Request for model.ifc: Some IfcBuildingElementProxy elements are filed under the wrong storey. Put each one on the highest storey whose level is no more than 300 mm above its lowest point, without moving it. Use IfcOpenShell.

First a look at what the model holds.

```python
import ifcopenshell
import ifcopenshell.util.element
import ifcopenshell.util.placement

model = ifcopenshell.open("model.ifc")
print(model.schema)
for storey in model.by_type("IfcBuildingStorey"):
    level = ifcopenshell.util.placement.get_storey_elevation(storey)
    count = sum(e.is_a("IfcBuildingElementProxy") for e in ifcopenshell.util.element.get_contained(storey))
    print(storey.id(), storey.Name, round(level, 3), count, sep=" | ")
```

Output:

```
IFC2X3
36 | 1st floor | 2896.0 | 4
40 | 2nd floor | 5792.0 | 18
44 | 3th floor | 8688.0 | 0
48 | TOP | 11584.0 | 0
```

```python
import ifcopenshell
import ifcopenshell.api.spatial
import ifcopenshell.geom
import ifcopenshell.util.element
import ifcopenshell.util.placement
import ifcopenshell.util.shape
import ifcopenshell.util.unit

model = ifcopenshell.open("model.ifc")
unit_scale = ifcopenshell.util.unit.calculate_unit_scale(model)
settings = ifcopenshell.geom.settings()

levels = sorted(
    ((ifcopenshell.util.placement.get_storey_elevation(s) * unit_scale, s) for s in model.by_type("IfcBuildingStorey")),
    key=lambda pair: pair[0],
)

for e in model.by_type("IfcBuildingElementProxy"):
    current = e.ContainedInStructure[0].RelatingStructure if e.ContainedInStructure else None
    if current is None or not current.is_a("IfcBuildingStorey"):
        continue
    shape = ifcopenshell.geom.create_shape(settings, e)
    bottom = ifcopenshell.util.shape.get_shape_bottom_elevation(shape, shape.geometry)
    below = [s for level, s in levels if level <= bottom + 0.3]
    storey = below[-1] if below else levels[0][1]
    if storey != current:
        # assign_container keeps the world position.
        ifcopenshell.api.spatial.assign_container(model, products=[e], relating_structure=storey)
        print(e.id(), current.Name, "->", storey.Name)

model.write("model_v2.ifc")
```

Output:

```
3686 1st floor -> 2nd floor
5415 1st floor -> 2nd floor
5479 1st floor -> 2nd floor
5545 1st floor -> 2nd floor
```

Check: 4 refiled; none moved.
